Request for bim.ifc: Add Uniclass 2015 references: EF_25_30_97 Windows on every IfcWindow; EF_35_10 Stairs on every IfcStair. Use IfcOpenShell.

First a look at what the model holds.

```python
import ifcopenshell

model = ifcopenshell.open("bim.ifc")
print(model.schema)
print("classifications:", [c.Name for c in model.by_type("IfcClassification")])
for ifc_class in ("IfcDoor", "IfcRoof", "IfcStair", "IfcWall", "IfcWindow"):
    print(ifc_class, len(model.by_type(ifc_class)))
```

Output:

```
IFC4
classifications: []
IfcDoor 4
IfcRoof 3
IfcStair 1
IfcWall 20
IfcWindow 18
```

```python
import ifcopenshell
import ifcopenshell.api.classification

model = ifcopenshell.open("bim.ifc")

system = ifcopenshell.api.classification.add_classification(model, classification="Uniclass 2015")

codes = {
    "IfcWindow": ("EF_25_30_97", "Windows"),
    "IfcStair": ("EF_35_10", "Stairs"),
}
for ifc_class, (code, name) in codes.items():
    products = model.by_type(ifc_class)
    ifcopenshell.api.classification.add_reference(
        model, products=products, classification=system, identification=code, name=name
    )
    print(code, len(products))

model.write("bim_rev.ifc")
```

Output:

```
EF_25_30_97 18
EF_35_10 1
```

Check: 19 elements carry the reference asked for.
